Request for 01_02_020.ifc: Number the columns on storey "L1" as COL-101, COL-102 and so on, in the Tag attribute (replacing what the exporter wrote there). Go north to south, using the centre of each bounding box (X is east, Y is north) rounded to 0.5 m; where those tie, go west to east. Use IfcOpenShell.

First a look at what the model holds.

```python
import ifcopenshell
import ifcopenshell.util.element
import ifcopenshell.util.placement

model = ifcopenshell.open("01_02_020.ifc")
print(model.schema)
storey = next(s for s in model.by_type("IfcBuildingStorey") if s.Name == "L1")
columns = [e for e in ifcopenshell.util.element.get_decomposition(storey) if e.is_a("IfcColumn")]
for e in sorted(columns, key=lambda e: e.id()):
    origin = ifcopenshell.util.placement.get_local_placement(e.ObjectPlacement)[:3, 3]
    print(e.id(), e.Tag, e.Name, origin.round(2) + 0.0, sep=" | ")
```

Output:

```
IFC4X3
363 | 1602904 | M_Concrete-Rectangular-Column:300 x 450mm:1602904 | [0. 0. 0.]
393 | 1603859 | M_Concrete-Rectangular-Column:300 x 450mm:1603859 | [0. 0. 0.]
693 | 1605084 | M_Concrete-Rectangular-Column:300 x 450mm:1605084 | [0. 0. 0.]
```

```python
import ifcopenshell
import ifcopenshell.geom
import ifcopenshell.util.element
import ifcopenshell.util.shape

model = ifcopenshell.open("01_02_020.ifc")
settings = ifcopenshell.geom.settings()
settings.set("use-world-coords", True)


def centre(element):
    shape = ifcopenshell.geom.create_shape(settings, element)
    return ifcopenshell.util.shape.get_bbox_centroid(shape.geometry)


storey = next(s for s in model.by_type("IfcBuildingStorey") if s.Name == "L1")
columns = [e for e in ifcopenshell.util.element.get_decomposition(storey) if e.is_a("IfcColumn")]

# Insertion points can sit at a corner or the storey origin, so sort by the geometry (in metres).
centres = {e: centre(e) for e in columns}
columns.sort(key=lambda e: (-round(centres[e][1] / 0.5), centres[e][0]))

for i, e in enumerate(columns, start=1):
    number = f"COL-1{i:02d}"
    e.Tag = number
    print(e.id(), number)

model.write("01_02_020-out.ifc")
```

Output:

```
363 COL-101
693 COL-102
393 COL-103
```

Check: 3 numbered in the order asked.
